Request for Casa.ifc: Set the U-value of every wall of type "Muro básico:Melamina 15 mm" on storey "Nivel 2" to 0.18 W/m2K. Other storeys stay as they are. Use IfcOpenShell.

First a look at what the model holds.

```python
import ifcopenshell
import ifcopenshell.util.element

model = ifcopenshell.open("Casa.ifc")
print(model.schema)
storey = next(s for s in model.by_type("IfcBuildingStorey") if s.Name == "Nivel 2")
walls = [e for e in ifcopenshell.util.element.get_decomposition(storey) if e.is_a("IfcWall")]
seen = {}
for e in walls:
    element_type = ifcopenshell.util.element.get_type(e)
    key = (element_type.Name if element_type != e and element_type else None, ifcopenshell.util.element.get_pset(e, "Pset_WallCommon", "ThermalTransmittance"))
    seen[key] = seen.get(key, 0) + 1
for (name, value), count in sorted(seen.items(), key=str):
    print(count, "x", name, "|", value)
```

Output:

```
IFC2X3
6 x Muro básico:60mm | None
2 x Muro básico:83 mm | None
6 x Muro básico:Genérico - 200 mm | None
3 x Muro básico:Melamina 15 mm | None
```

```python
import ifcopenshell
import ifcopenshell.api.pset
import ifcopenshell.util.element

model = ifcopenshell.open("Casa.ifc")

storey = next(s for s in model.by_type("IfcBuildingStorey") if s.Name == "Nivel 2")
walls = [e for e in ifcopenshell.util.element.get_decomposition(storey) if e.is_a("IfcWall")]

count = 0
for e in walls:
    element_type = ifcopenshell.util.element.get_type(e)
    if element_type in (None, e) or element_type.Name != "Muro básico:Melamina 15 mm":
        continue
    # add_pset returns the element's existing set when there is one.
    pset = ifcopenshell.api.pset.add_pset(model, product=e, name="Pset_WallCommon")
    ifcopenshell.api.pset.edit_pset(model, pset=pset, properties={"ThermalTransmittance": 0.18})
    count += 1

print(count, "walls updated")

model.write("Casa_v2.ifc")
```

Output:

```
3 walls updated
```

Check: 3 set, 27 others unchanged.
